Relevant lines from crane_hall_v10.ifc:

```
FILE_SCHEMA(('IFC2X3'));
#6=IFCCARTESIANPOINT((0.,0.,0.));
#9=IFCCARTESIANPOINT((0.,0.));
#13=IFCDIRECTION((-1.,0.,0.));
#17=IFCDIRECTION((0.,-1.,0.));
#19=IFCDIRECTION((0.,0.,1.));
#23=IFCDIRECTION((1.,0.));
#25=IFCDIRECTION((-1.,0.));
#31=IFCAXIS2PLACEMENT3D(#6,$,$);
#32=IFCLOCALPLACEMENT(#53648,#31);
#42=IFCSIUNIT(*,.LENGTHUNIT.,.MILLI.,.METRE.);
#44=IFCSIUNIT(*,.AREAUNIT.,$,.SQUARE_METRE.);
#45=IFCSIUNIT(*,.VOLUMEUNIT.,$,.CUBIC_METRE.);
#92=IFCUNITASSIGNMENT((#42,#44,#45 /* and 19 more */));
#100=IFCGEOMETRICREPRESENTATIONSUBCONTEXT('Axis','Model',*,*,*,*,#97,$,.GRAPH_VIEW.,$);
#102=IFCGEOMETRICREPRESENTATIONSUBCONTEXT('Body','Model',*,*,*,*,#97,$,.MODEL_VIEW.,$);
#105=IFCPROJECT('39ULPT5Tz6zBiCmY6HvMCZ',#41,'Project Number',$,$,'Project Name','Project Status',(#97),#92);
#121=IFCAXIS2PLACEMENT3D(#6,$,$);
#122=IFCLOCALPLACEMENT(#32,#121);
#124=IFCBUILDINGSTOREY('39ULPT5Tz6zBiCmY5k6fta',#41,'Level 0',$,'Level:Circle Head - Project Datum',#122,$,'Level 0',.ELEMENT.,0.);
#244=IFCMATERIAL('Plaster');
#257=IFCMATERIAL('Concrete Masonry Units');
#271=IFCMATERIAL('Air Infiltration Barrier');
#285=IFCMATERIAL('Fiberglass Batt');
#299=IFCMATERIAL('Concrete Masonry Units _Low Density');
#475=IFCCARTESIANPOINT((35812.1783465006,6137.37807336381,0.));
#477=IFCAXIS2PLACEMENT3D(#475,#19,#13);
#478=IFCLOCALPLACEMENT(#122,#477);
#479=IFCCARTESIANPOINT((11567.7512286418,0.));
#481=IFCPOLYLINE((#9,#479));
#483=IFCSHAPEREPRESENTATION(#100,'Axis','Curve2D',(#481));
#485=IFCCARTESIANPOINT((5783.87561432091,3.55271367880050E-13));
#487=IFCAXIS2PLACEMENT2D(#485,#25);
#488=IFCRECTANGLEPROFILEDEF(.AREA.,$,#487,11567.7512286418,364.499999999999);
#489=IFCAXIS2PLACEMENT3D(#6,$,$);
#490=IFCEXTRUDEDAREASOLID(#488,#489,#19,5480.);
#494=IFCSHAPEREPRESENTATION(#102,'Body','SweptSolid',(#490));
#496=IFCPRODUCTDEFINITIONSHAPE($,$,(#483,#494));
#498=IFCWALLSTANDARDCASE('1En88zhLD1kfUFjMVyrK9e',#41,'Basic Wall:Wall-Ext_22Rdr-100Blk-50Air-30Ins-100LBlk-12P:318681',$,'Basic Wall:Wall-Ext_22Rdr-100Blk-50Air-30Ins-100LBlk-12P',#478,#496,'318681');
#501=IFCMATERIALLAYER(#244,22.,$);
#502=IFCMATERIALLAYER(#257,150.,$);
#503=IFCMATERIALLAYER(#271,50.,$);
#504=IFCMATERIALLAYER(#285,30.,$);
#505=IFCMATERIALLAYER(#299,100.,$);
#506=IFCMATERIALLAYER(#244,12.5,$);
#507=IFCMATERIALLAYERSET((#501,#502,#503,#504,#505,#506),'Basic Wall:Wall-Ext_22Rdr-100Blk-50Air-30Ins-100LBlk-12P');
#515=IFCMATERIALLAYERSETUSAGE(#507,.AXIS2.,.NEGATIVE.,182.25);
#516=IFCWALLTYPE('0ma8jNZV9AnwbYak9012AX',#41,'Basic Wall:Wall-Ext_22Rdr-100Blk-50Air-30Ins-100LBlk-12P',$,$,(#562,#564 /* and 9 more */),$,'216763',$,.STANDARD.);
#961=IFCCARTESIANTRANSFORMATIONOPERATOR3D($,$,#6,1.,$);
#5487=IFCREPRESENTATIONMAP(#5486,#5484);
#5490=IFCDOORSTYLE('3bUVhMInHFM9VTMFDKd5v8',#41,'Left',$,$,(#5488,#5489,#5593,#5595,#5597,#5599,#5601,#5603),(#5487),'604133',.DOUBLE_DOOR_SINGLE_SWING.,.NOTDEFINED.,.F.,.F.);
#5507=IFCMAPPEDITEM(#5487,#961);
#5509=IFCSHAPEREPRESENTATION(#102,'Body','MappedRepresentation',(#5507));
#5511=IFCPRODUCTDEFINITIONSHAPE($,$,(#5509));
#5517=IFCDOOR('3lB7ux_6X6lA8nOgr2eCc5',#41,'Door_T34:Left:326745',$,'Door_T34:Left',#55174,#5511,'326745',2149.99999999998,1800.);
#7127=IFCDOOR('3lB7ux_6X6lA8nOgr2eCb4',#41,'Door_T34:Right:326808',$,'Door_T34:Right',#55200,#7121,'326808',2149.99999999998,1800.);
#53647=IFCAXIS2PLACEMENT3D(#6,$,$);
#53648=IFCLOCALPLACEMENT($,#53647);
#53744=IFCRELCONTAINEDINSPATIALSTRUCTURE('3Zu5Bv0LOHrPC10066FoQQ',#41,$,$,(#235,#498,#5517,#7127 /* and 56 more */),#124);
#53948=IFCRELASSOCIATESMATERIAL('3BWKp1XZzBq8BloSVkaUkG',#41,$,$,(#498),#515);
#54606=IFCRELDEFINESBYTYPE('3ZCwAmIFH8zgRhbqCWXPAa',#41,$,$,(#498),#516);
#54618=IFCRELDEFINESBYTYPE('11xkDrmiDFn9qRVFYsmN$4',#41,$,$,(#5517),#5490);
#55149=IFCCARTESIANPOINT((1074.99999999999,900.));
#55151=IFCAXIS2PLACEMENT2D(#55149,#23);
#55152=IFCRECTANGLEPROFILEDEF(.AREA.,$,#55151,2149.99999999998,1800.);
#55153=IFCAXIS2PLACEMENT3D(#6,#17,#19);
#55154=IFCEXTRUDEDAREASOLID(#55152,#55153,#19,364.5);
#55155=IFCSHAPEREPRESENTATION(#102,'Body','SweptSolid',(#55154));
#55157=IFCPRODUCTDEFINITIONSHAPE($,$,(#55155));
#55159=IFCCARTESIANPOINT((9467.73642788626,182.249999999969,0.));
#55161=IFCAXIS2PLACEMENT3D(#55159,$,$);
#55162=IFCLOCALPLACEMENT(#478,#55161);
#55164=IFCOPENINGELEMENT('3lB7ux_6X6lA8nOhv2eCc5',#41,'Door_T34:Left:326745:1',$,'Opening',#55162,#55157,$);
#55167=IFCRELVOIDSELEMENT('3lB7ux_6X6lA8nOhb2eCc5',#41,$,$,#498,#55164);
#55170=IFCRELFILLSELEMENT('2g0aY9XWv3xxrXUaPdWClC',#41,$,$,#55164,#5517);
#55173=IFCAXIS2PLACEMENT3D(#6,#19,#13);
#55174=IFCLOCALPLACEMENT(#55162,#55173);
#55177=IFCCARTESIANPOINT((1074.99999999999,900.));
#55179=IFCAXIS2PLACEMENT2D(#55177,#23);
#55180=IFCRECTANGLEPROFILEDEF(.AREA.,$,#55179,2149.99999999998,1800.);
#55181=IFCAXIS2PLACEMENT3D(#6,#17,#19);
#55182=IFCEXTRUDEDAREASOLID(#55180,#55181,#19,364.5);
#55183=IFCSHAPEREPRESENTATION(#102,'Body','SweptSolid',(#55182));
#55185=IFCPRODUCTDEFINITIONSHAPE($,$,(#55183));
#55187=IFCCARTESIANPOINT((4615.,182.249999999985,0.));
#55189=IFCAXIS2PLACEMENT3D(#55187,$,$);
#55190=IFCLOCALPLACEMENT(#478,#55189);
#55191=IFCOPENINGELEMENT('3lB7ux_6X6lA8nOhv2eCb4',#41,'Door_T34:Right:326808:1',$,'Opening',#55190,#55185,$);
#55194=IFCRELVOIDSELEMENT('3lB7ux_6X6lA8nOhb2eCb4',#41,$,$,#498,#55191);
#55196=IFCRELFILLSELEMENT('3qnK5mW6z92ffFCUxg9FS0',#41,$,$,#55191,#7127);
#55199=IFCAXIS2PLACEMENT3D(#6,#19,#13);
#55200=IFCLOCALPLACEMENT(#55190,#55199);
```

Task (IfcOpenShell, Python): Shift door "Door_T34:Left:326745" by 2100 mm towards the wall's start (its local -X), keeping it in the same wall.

```python
import ifcopenshell
import ifcopenshell.api.geometry
import ifcopenshell.util.placement
import ifcopenshell.util.unit

model = ifcopenshell.open("crane_hall_v10.ifc")
unit_scale = ifcopenshell.util.unit.calculate_unit_scale(model)

door = model.by_id(5517)
opening = door.FillsVoids[0].RelatingOpeningElement
wall = opening.VoidsElements[0].RelatingBuildingElement

wall_matrix = ifcopenshell.util.placement.get_local_placement(wall.ObjectPlacement)
shift = wall_matrix[:3, 0] * -2.1 / unit_scale
before = ifcopenshell.util.placement.get_local_placement(door.ObjectPlacement)[:3, 3].copy()

# The door is placed relative to its opening, so it follows when the opening moves.
matrix = ifcopenshell.util.placement.get_local_placement(opening.ObjectPlacement)
matrix[:3, 3] += shift
ifcopenshell.api.geometry.edit_object_placement(
    model, product=opening, matrix=matrix, is_si=False, should_transform_children=True
)

after = ifcopenshell.util.placement.get_local_placement(door.ObjectPlacement)[:3, 3]
print("door moved by", (after - before).round(3) + 0.0)

model.write("crane_hall_v10_updated.ifc")
```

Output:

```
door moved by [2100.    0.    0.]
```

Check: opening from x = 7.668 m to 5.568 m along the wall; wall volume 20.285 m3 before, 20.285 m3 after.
